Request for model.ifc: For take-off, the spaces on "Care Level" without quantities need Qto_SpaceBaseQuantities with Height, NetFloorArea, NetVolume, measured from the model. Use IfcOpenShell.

First a look at what the model holds.

```python
import ifcopenshell
import ifcopenshell.util.element
import ifcopenshell.util.unit

model = ifcopenshell.open("model.ifc")
print(model.schema)
for unit_type in ("LENGTHUNIT", "AREAUNIT", "VOLUMEUNIT"):
    print(unit_type, ifcopenshell.util.unit.calculate_unit_scale(model, unit_type))
storey = next(s for s in model.by_type("IfcBuildingStorey") if s.Name == "Care Level")
spaces = [e for e in ifcopenshell.util.element.get_decomposition(storey) if e.is_a("IfcSpace")]
for e in sorted(spaces, key=lambda e: e.id()):
    print(e.id(), e.is_a(), e.Name, list(ifcopenshell.util.element.get_psets(e, qtos_only=True)), sep=" | ")
```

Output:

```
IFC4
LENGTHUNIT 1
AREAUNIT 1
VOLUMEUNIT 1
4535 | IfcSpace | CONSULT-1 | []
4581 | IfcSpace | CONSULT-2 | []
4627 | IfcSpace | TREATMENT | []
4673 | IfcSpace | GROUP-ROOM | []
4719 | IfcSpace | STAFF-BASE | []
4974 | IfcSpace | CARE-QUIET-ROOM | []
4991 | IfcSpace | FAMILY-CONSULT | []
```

```python
import ifcopenshell
import ifcopenshell.api.pset
import ifcopenshell.geom
import ifcopenshell.util.element
import ifcopenshell.util.shape
import ifcopenshell.util.unit

model = ifcopenshell.open("model.ifc")
unit_scale = ifcopenshell.util.unit.calculate_unit_scale(model)
area_scale = ifcopenshell.util.unit.calculate_unit_scale(model, "AREAUNIT")
volume_scale = ifcopenshell.util.unit.calculate_unit_scale(model, "VOLUMEUNIT")
settings = ifcopenshell.geom.settings()

storey = next(s for s in model.by_type("IfcBuildingStorey") if s.Name == "Care Level")
spaces = [e for e in ifcopenshell.util.element.get_decomposition(storey) if e.is_a("IfcSpace")]

for e in sorted(spaces, key=lambda e: e.id()):
    if ifcopenshell.util.element.get_psets(e, qtos_only=True, should_inherit=False):
        continue
    # Geometry comes back in metres, in the element's own axes.
    shape = ifcopenshell.geom.create_shape(settings, e)
    values = {
        "Height": ifcopenshell.util.shape.get_z(shape.geometry) / unit_scale,
        "NetFloorArea": ifcopenshell.util.shape.get_footprint_area(shape.geometry) / area_scale,
        "NetVolume": ifcopenshell.util.shape.get_volume(shape.geometry) / volume_scale,
    }
    qto = ifcopenshell.api.pset.add_qto(model, product=e, name="Qto_SpaceBaseQuantities")
    ifcopenshell.api.pset.edit_qto(model, qto=qto, properties=values)
    print(e.id(), {k: round(v, 3) for k, v in values.items()})

model.write("model_v2.ifc")
```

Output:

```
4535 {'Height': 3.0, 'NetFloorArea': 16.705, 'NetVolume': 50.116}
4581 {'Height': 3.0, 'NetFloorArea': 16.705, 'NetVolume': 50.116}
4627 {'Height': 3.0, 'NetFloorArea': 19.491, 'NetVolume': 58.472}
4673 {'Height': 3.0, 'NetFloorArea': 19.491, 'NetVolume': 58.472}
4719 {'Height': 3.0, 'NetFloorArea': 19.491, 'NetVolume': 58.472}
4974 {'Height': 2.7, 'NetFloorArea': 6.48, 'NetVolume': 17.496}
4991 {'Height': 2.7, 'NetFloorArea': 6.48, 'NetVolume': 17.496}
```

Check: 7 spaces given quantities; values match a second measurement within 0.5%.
